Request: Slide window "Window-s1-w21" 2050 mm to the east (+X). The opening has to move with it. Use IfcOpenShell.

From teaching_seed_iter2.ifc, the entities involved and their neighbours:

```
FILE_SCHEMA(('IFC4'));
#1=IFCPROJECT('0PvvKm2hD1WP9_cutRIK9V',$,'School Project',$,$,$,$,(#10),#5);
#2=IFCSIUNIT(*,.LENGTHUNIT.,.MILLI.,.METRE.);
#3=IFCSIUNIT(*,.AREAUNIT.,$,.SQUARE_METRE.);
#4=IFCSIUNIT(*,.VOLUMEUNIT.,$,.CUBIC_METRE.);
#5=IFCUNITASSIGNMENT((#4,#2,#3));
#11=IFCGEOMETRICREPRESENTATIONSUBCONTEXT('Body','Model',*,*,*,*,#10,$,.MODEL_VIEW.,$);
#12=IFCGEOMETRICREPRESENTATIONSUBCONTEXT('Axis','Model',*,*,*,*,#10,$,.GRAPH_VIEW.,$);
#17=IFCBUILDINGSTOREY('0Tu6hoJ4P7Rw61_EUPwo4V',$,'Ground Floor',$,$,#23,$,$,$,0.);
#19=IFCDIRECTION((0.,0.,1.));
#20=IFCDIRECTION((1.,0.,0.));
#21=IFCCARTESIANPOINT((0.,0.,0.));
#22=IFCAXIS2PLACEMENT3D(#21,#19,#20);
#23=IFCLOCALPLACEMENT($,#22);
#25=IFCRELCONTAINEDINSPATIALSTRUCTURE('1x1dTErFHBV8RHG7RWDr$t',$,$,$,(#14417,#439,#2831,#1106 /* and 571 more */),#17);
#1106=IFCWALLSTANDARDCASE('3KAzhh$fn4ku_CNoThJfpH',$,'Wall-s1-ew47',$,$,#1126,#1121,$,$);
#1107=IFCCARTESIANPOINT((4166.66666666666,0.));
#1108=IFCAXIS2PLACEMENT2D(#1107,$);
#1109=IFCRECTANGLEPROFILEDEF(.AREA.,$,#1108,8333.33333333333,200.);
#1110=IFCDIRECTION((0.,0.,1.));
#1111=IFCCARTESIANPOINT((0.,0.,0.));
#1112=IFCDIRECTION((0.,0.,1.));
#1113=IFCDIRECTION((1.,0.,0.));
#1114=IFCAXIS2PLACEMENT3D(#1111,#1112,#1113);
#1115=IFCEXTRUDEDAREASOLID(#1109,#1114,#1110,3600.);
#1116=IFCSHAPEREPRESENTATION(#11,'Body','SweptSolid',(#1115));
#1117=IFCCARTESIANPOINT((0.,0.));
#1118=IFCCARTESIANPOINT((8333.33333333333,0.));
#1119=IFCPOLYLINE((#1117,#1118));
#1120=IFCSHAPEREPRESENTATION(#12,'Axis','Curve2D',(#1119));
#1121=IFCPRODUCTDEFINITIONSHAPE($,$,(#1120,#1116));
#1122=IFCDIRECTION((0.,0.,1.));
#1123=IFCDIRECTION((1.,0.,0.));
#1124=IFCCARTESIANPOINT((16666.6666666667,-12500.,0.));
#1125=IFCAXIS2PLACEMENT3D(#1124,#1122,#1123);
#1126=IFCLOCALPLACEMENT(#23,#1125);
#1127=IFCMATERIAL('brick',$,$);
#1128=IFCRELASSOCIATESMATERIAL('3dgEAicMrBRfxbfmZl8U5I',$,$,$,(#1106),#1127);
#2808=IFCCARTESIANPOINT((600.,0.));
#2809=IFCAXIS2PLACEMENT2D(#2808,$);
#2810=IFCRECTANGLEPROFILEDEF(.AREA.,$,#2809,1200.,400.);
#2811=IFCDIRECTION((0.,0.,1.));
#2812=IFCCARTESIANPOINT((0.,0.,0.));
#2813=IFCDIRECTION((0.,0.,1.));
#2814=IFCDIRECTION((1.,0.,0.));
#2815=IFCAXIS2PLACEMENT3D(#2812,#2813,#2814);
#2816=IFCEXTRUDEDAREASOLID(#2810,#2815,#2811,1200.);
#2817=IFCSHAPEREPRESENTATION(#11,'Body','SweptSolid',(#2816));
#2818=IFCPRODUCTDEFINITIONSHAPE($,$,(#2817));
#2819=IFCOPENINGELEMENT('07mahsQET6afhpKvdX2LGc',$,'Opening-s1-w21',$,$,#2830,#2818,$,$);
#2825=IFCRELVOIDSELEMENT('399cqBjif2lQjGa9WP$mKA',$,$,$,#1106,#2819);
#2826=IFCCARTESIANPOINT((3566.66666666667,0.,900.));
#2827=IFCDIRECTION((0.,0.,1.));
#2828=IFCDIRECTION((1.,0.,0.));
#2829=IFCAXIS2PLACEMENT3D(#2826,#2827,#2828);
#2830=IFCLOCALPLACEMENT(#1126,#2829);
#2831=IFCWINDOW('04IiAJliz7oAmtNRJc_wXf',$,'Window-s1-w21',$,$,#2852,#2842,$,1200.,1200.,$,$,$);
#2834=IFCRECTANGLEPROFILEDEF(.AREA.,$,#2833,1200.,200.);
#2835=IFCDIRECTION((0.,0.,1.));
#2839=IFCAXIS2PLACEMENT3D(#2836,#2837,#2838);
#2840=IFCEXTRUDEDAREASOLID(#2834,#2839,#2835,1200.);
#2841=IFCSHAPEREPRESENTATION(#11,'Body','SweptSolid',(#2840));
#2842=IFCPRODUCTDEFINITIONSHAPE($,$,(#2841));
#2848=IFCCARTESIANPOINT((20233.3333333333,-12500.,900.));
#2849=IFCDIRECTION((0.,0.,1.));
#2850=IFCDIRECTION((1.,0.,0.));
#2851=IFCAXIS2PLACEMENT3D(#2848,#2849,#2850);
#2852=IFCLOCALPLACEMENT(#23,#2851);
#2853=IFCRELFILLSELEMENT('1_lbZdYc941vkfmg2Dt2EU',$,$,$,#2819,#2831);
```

```python
import ifcopenshell
import ifcopenshell.api.geometry
import ifcopenshell.util.placement
import ifcopenshell.util.unit

model = ifcopenshell.open("teaching_seed_iter2.ifc")
unit_scale = ifcopenshell.util.unit.calculate_unit_scale(model)

window = model.by_id(2831)
opening = window.FillsVoids[0].RelatingOpeningElement
wall = opening.VoidsElements[0].RelatingBuildingElement

wall_matrix = ifcopenshell.util.placement.get_local_placement(wall.ObjectPlacement)
shift = wall_matrix[:3, 0] * 2.05 / unit_scale
before = ifcopenshell.util.placement.get_local_placement(window.ObjectPlacement)[:3, 3].copy()

# The window is not placed relative to its opening, so move both.
for product in (opening, window):
    matrix = ifcopenshell.util.placement.get_local_placement(product.ObjectPlacement)
    matrix[:3, 3] += shift
    ifcopenshell.api.geometry.edit_object_placement(model, product=product, matrix=matrix, is_si=False)

after = ifcopenshell.util.placement.get_local_placement(window.ObjectPlacement)[:3, 3]
print("window moved by", (after - before).round(3) + 0.0)

model.write("teaching_seed_iter2_v2.ifc")
```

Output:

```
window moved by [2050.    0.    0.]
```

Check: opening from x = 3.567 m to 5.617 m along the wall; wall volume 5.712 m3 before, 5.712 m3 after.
